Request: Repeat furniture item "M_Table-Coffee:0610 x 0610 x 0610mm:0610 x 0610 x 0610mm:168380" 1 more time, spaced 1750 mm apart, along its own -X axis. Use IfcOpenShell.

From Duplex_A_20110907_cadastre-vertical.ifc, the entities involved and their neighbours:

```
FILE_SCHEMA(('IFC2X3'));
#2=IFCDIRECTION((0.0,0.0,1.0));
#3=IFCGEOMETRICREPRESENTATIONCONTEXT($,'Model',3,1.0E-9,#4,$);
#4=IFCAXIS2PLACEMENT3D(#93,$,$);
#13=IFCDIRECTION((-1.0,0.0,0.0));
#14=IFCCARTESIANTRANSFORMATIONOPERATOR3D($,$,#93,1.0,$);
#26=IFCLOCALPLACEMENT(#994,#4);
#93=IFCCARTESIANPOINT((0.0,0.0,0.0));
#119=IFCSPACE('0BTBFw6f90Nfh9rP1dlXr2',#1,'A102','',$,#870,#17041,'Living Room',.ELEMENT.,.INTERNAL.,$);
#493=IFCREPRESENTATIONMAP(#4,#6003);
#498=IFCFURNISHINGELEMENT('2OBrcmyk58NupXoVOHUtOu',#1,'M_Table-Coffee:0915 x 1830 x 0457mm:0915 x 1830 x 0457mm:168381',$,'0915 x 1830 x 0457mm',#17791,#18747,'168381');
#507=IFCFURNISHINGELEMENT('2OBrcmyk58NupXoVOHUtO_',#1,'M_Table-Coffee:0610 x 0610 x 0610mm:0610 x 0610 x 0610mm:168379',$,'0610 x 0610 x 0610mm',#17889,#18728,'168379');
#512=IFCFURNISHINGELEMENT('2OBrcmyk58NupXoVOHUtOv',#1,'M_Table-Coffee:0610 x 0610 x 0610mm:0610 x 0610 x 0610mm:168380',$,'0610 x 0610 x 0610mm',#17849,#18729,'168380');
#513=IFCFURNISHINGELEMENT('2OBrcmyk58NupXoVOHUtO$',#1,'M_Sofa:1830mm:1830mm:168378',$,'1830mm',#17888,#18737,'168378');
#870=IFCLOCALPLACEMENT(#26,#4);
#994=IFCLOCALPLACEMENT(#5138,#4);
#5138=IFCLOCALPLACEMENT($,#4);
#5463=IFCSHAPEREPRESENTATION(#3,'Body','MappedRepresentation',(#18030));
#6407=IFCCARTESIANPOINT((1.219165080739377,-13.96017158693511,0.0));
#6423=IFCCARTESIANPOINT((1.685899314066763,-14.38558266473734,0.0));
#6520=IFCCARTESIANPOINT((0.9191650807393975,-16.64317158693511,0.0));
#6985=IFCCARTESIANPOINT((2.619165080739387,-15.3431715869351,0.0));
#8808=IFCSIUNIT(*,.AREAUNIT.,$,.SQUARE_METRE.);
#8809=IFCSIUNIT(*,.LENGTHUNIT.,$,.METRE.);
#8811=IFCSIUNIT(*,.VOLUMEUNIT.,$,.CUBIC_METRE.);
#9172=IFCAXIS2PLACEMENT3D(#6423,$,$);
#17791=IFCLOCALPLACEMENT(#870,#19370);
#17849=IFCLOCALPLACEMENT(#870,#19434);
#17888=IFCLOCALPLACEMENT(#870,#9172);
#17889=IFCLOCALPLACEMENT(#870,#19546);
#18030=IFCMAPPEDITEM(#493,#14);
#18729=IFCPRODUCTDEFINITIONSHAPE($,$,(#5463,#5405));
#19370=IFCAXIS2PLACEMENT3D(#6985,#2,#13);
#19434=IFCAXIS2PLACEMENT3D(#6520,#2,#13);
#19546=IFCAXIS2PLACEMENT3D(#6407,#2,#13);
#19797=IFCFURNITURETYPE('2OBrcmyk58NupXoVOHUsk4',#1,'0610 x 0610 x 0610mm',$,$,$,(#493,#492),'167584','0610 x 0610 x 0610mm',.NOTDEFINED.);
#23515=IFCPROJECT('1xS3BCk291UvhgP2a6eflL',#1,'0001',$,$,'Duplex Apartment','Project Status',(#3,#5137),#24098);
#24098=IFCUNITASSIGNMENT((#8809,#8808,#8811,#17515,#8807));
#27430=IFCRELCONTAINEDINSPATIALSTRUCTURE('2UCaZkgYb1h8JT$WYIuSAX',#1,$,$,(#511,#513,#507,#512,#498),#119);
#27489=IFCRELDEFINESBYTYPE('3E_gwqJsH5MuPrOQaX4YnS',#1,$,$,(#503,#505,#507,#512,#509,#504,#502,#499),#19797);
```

```python
import ifcopenshell
import ifcopenshell.api.geometry
import ifcopenshell.api.root
import ifcopenshell.util.element
import ifcopenshell.util.placement
import ifcopenshell.util.unit

model = ifcopenshell.open("Duplex_A_20110907_cadastre-vertical.ifc")
unit_scale = ifcopenshell.util.unit.calculate_unit_scale(model)


def reuse_history(source, copy):
    """copy_class also copies each property set's owner history, people and application; keep the originals."""
    for rel in copy.IsDefinedBy:
        if rel.is_a("IfcRelDefinesByProperties") and (history := rel.RelatingPropertyDefinition.OwnerHistory):
            rel.RelatingPropertyDefinition.OwnerHistory = source.OwnerHistory
            ifcopenshell.util.element.remove_deep2(model, history)


source = model.by_id(512)
base = ifcopenshell.util.placement.get_local_placement(source.ObjectPlacement)
step = -base[:3, 0] * 1.75 / unit_scale

for i in range(1, 2):
    copy = ifcopenshell.api.root.copy_class(model, product=source)
    copy.Representation = ifcopenshell.util.element.copy_deep(
        model, source.Representation, exclude=["IfcGeometricRepresentationContext", "IfcRepresentationMap"]
    )
    copy.Name = "M_Table-Coffee:0610 x 0610 x 0610mm:0610 x 0610 x 0610mm"
    copy.Tag = None
    reuse_history(source, copy)
    matrix = base.copy()
    matrix[:3, 3] += i * step
    print("added at", matrix[:3, 3].round(3) + 0.0)
    ifcopenshell.api.geometry.edit_object_placement(model, product=copy, matrix=matrix, is_si=False)

model.write("Duplex_A_20110907_cadastre-vertical_updated.ifc")
```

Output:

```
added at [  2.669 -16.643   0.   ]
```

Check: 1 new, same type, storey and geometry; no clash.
